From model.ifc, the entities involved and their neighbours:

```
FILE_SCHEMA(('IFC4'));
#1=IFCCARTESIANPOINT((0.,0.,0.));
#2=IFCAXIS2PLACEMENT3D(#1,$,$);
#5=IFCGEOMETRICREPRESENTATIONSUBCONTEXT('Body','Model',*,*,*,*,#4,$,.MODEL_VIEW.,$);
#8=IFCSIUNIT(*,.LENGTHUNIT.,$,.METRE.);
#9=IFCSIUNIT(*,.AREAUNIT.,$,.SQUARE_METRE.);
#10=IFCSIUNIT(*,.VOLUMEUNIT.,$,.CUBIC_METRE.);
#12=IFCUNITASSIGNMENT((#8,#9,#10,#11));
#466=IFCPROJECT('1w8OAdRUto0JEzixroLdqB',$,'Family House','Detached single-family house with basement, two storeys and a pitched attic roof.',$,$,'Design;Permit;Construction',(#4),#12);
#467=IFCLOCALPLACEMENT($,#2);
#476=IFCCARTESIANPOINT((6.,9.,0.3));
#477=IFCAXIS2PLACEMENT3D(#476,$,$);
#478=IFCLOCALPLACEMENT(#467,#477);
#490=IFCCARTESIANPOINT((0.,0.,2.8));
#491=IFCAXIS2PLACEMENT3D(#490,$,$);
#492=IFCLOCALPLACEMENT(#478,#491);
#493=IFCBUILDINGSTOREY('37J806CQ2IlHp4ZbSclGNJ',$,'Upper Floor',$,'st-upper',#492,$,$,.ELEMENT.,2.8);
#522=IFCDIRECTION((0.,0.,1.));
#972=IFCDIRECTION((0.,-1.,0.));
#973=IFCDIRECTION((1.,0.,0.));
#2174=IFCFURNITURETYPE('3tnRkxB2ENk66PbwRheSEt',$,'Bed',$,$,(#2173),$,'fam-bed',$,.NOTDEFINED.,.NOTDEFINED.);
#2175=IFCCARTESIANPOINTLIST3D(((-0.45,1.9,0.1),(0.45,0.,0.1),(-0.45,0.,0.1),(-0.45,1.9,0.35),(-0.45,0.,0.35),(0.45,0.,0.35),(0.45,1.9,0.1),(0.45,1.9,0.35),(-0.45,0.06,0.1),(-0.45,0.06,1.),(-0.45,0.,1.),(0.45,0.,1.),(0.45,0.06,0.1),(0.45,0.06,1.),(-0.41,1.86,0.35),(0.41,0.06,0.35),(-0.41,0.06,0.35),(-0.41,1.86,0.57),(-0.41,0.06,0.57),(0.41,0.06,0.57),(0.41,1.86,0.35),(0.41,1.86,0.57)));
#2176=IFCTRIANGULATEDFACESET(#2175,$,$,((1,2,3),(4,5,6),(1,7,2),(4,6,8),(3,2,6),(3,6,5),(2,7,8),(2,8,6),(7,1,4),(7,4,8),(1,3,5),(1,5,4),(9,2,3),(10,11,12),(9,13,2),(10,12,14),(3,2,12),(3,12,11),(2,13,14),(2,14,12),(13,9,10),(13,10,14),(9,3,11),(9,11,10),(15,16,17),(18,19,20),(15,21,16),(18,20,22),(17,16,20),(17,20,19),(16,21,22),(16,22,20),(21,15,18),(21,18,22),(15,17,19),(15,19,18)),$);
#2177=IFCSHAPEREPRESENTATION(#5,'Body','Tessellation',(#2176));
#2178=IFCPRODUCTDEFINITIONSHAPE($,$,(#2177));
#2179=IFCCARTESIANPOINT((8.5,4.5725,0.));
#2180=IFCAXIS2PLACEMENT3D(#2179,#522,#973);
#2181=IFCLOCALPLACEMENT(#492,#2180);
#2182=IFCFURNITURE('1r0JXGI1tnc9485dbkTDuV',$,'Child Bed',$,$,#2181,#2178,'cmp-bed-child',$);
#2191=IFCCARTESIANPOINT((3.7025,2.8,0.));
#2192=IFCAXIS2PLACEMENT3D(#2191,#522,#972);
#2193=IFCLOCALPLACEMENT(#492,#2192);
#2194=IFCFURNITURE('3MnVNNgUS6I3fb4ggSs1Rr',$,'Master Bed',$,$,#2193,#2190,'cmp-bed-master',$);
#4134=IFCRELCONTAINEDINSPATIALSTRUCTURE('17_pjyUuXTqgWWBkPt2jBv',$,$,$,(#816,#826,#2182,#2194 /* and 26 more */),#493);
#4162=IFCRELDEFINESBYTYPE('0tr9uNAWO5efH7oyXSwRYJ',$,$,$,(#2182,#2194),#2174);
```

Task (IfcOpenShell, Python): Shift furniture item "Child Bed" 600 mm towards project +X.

```python
import ifcopenshell
import ifcopenshell.api.geometry
import ifcopenshell.util.placement
import ifcopenshell.util.unit

model = ifcopenshell.open("model.ifc")
unit_scale = ifcopenshell.util.unit.calculate_unit_scale(model)

item = model.by_id(2182)
matrix = ifcopenshell.util.placement.get_local_placement(item.ObjectPlacement)
matrix[0, 3] += 0.6 / unit_scale
ifcopenshell.api.geometry.edit_object_placement(model, product=item, matrix=matrix, is_si=False)

print(ifcopenshell.util.placement.get_local_placement(item.ObjectPlacement).round(3) + 0.0)

model.write("model-out.ifc")
```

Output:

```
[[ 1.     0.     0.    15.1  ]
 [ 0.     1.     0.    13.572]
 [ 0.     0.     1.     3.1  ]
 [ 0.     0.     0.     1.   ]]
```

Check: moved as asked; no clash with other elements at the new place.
